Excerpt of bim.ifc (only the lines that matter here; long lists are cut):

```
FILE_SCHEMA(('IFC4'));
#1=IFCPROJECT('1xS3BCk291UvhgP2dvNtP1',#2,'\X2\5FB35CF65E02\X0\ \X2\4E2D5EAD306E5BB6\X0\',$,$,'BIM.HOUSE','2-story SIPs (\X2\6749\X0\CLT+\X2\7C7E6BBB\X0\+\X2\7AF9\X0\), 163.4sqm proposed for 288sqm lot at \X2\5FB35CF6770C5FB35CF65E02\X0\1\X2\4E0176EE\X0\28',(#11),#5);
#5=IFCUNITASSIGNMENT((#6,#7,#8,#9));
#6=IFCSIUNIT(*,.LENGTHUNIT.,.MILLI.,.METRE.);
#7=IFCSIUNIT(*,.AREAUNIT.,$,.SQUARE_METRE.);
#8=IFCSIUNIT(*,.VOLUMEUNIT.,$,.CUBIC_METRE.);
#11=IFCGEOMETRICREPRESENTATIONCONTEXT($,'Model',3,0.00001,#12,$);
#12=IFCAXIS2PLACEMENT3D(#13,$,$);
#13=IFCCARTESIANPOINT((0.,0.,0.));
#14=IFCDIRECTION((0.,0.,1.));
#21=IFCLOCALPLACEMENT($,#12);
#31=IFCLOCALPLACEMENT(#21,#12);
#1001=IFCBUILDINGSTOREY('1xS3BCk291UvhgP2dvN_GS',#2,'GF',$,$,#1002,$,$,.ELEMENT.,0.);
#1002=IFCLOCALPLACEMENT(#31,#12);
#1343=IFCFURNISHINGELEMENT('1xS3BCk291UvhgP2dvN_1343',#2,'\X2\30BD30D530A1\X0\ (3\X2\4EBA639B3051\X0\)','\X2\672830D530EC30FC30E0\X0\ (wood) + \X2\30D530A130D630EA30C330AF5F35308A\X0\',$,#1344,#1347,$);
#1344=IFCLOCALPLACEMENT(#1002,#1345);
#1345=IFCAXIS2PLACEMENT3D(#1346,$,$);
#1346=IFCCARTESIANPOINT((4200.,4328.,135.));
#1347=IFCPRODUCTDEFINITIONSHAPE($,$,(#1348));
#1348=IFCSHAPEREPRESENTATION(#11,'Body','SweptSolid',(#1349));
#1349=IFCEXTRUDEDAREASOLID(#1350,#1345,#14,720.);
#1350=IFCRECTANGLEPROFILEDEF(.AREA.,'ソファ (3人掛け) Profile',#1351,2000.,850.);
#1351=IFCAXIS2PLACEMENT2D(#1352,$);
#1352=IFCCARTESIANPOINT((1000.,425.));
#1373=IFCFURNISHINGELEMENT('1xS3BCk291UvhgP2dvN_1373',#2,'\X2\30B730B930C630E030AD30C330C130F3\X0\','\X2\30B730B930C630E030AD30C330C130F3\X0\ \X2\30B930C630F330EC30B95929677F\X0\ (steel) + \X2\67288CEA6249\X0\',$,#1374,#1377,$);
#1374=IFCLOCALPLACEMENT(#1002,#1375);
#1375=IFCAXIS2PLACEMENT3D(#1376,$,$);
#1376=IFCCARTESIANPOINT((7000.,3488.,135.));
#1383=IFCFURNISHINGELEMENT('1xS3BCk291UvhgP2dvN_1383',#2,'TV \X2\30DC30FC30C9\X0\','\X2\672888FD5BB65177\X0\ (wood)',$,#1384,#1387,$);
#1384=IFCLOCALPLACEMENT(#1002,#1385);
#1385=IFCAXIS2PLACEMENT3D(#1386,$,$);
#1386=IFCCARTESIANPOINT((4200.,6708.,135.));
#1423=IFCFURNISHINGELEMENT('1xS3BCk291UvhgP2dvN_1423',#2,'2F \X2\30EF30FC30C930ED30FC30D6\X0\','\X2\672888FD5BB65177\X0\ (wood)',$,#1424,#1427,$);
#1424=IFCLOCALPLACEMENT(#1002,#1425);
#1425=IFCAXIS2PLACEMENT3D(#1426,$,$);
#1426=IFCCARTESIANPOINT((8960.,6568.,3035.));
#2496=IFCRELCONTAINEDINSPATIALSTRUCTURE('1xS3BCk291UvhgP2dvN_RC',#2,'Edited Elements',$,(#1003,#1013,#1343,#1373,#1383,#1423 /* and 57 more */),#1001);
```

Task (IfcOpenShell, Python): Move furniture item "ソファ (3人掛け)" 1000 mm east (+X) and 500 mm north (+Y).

```python
import ifcopenshell
import ifcopenshell.api.geometry
import ifcopenshell.util.placement
import ifcopenshell.util.unit

model = ifcopenshell.open("bim.ifc")
unit_scale = ifcopenshell.util.unit.calculate_unit_scale(model)

item = model.by_id(1343)
matrix = ifcopenshell.util.placement.get_local_placement(item.ObjectPlacement)
matrix[0, 3] += 1 / unit_scale
matrix[1, 3] += 0.5 / unit_scale
ifcopenshell.api.geometry.edit_object_placement(model, product=item, matrix=matrix, is_si=False)

print(ifcopenshell.util.placement.get_local_placement(item.ObjectPlacement).round(3) + 0.0)

model.write("bim_rev.ifc")
```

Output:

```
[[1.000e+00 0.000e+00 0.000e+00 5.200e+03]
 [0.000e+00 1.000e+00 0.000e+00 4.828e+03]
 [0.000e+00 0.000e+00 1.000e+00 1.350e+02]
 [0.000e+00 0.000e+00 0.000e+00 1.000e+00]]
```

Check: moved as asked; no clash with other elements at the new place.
